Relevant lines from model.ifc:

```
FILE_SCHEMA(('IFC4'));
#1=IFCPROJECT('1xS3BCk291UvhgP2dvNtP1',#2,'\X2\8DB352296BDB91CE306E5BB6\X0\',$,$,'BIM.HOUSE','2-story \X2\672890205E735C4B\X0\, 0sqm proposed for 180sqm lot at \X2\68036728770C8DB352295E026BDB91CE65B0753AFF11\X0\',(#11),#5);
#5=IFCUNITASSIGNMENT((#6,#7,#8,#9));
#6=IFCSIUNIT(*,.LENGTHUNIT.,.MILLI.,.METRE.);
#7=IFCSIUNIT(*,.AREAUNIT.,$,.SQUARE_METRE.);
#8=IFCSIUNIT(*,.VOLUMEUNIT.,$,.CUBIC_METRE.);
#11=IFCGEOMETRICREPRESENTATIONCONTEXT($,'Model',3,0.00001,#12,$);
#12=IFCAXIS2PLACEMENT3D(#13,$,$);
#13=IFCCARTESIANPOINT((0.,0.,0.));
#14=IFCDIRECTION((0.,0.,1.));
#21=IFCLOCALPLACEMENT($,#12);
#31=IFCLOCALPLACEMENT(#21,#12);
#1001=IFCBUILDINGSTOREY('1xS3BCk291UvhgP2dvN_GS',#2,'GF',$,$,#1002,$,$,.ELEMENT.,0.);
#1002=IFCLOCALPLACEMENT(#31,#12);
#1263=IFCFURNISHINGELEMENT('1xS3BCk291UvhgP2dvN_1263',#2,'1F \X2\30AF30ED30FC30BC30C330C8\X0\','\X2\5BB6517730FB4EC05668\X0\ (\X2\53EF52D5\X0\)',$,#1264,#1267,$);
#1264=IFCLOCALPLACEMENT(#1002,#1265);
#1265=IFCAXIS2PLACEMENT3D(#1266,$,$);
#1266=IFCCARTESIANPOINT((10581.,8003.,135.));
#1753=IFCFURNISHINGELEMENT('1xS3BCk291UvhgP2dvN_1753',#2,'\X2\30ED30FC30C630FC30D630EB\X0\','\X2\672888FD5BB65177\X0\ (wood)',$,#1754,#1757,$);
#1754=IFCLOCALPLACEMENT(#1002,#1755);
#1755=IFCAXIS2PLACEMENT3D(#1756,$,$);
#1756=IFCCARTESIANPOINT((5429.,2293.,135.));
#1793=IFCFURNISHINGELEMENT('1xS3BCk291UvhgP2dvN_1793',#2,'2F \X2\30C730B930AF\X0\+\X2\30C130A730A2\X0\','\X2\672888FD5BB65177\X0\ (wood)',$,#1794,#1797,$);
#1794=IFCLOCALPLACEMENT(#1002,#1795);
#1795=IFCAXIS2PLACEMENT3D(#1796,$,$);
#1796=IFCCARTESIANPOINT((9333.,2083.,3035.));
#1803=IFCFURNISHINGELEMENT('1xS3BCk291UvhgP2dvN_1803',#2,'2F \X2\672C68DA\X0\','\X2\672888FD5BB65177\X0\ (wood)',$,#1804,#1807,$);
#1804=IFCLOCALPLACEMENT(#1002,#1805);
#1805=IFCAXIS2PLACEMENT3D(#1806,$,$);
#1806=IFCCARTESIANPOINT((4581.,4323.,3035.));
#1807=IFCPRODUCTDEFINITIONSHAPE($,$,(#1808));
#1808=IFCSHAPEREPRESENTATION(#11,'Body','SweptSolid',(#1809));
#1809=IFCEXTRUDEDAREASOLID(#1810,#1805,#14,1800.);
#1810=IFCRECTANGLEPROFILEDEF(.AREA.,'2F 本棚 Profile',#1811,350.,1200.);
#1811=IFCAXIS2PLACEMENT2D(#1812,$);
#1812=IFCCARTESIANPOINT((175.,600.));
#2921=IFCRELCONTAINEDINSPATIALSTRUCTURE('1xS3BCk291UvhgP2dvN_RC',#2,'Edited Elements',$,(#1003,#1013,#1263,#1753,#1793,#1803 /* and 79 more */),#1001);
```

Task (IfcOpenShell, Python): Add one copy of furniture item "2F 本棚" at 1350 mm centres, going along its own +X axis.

```python
import ifcopenshell
import ifcopenshell.api.geometry
import ifcopenshell.api.root
import ifcopenshell.util.element
import ifcopenshell.util.placement

model = ifcopenshell.open("model.ifc")


def reuse_history(source, copy):
    """copy_class also copies each property set's owner history, people and application; keep the originals."""
    for rel in copy.IsDefinedBy:
        if rel.is_a("IfcRelDefinesByProperties") and (history := rel.RelatingPropertyDefinition.OwnerHistory):
            rel.RelatingPropertyDefinition.OwnerHistory = source.OwnerHistory
            ifcopenshell.util.element.remove_deep2(model, history)


source = model.by_id(1803)
base = ifcopenshell.util.placement.get_local_placement(source.ObjectPlacement)
step = base[:3, 0] * 1350.0

for i in range(1, 2):
    copy = ifcopenshell.api.root.copy_class(model, product=source)
    copy.Representation = ifcopenshell.util.element.copy_deep(
        model, source.Representation, exclude=["IfcGeometricRepresentationContext", "IfcRepresentationMap"]
    )
    reuse_history(source, copy)
    matrix = base.copy()
    matrix[:3, 3] += i * step
    print("added at", matrix[:3, 3].round(3) + 0.0)
    ifcopenshell.api.geometry.edit_object_placement(model, product=copy, matrix=matrix, is_si=False)

model.write("model_updated.ifc")
```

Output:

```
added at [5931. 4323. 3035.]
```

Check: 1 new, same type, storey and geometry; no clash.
